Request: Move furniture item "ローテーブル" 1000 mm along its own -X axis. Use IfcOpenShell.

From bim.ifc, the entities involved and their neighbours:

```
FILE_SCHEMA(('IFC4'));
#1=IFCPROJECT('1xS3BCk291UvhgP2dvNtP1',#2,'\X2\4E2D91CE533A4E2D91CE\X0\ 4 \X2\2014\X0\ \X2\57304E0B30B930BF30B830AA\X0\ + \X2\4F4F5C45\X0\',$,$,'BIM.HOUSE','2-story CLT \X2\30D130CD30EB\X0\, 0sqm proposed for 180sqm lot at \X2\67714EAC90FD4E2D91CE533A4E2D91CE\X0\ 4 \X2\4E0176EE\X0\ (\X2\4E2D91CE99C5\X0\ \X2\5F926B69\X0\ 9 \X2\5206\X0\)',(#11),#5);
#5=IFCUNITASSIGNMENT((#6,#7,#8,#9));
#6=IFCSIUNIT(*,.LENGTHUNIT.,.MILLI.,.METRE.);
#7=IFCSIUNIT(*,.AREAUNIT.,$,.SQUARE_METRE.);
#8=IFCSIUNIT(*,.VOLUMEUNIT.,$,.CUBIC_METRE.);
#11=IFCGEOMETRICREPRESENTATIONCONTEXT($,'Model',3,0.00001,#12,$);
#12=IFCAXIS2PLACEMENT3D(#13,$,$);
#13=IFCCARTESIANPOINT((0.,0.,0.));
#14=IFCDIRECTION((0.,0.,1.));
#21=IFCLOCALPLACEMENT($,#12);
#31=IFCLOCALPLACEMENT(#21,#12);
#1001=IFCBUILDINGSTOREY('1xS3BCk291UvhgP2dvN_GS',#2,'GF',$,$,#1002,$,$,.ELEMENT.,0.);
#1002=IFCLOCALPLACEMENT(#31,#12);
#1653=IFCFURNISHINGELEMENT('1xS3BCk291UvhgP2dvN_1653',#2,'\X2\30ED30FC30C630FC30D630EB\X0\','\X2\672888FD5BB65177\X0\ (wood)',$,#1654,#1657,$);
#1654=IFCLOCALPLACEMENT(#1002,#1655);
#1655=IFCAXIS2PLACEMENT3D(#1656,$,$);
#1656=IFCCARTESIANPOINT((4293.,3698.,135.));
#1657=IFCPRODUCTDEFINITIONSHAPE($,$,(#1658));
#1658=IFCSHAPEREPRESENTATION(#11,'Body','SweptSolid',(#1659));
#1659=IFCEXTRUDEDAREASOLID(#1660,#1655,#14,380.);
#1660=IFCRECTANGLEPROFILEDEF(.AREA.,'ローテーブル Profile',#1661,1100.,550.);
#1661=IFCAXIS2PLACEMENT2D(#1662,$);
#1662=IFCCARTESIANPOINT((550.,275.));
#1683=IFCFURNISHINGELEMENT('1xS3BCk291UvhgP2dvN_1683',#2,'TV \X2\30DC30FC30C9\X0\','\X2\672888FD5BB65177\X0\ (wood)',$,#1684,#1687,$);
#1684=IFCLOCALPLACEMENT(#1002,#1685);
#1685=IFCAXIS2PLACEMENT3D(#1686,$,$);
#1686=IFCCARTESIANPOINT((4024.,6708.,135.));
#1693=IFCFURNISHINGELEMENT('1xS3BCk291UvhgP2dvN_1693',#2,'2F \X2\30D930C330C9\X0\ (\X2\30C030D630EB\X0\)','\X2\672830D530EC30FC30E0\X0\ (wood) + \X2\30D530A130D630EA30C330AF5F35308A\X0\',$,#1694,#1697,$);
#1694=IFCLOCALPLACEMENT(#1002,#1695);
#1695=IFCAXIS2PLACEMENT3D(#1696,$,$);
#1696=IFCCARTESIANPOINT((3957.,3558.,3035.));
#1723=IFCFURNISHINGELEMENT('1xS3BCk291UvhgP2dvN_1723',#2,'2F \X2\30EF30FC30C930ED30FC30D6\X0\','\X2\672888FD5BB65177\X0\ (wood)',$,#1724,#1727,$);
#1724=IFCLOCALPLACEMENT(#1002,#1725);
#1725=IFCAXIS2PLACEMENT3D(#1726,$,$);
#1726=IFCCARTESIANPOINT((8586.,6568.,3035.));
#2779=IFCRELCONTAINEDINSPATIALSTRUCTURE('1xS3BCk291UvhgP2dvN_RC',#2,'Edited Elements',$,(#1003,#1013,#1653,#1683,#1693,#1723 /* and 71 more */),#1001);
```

```python
import ifcopenshell
import ifcopenshell.api.geometry
import ifcopenshell.util.placement
import ifcopenshell.util.unit

model = ifcopenshell.open("bim.ifc")
unit_scale = ifcopenshell.util.unit.calculate_unit_scale(model)

item = model.by_guid("1xS3BCk291UvhgP2dvN_1653")
matrix = ifcopenshell.util.placement.get_local_placement(item.ObjectPlacement)
matrix[:3, 3] -= matrix[:3, 0] * 1 / unit_scale
ifcopenshell.api.geometry.edit_object_placement(model, product=item, matrix=matrix, is_si=False)

print(ifcopenshell.util.placement.get_local_placement(item.ObjectPlacement).round(3) + 0.0)

model.write("bim_edited.ifc")
```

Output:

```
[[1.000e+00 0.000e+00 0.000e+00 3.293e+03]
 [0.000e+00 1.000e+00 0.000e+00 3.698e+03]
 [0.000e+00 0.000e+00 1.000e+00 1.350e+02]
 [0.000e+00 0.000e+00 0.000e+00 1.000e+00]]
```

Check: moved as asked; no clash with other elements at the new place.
